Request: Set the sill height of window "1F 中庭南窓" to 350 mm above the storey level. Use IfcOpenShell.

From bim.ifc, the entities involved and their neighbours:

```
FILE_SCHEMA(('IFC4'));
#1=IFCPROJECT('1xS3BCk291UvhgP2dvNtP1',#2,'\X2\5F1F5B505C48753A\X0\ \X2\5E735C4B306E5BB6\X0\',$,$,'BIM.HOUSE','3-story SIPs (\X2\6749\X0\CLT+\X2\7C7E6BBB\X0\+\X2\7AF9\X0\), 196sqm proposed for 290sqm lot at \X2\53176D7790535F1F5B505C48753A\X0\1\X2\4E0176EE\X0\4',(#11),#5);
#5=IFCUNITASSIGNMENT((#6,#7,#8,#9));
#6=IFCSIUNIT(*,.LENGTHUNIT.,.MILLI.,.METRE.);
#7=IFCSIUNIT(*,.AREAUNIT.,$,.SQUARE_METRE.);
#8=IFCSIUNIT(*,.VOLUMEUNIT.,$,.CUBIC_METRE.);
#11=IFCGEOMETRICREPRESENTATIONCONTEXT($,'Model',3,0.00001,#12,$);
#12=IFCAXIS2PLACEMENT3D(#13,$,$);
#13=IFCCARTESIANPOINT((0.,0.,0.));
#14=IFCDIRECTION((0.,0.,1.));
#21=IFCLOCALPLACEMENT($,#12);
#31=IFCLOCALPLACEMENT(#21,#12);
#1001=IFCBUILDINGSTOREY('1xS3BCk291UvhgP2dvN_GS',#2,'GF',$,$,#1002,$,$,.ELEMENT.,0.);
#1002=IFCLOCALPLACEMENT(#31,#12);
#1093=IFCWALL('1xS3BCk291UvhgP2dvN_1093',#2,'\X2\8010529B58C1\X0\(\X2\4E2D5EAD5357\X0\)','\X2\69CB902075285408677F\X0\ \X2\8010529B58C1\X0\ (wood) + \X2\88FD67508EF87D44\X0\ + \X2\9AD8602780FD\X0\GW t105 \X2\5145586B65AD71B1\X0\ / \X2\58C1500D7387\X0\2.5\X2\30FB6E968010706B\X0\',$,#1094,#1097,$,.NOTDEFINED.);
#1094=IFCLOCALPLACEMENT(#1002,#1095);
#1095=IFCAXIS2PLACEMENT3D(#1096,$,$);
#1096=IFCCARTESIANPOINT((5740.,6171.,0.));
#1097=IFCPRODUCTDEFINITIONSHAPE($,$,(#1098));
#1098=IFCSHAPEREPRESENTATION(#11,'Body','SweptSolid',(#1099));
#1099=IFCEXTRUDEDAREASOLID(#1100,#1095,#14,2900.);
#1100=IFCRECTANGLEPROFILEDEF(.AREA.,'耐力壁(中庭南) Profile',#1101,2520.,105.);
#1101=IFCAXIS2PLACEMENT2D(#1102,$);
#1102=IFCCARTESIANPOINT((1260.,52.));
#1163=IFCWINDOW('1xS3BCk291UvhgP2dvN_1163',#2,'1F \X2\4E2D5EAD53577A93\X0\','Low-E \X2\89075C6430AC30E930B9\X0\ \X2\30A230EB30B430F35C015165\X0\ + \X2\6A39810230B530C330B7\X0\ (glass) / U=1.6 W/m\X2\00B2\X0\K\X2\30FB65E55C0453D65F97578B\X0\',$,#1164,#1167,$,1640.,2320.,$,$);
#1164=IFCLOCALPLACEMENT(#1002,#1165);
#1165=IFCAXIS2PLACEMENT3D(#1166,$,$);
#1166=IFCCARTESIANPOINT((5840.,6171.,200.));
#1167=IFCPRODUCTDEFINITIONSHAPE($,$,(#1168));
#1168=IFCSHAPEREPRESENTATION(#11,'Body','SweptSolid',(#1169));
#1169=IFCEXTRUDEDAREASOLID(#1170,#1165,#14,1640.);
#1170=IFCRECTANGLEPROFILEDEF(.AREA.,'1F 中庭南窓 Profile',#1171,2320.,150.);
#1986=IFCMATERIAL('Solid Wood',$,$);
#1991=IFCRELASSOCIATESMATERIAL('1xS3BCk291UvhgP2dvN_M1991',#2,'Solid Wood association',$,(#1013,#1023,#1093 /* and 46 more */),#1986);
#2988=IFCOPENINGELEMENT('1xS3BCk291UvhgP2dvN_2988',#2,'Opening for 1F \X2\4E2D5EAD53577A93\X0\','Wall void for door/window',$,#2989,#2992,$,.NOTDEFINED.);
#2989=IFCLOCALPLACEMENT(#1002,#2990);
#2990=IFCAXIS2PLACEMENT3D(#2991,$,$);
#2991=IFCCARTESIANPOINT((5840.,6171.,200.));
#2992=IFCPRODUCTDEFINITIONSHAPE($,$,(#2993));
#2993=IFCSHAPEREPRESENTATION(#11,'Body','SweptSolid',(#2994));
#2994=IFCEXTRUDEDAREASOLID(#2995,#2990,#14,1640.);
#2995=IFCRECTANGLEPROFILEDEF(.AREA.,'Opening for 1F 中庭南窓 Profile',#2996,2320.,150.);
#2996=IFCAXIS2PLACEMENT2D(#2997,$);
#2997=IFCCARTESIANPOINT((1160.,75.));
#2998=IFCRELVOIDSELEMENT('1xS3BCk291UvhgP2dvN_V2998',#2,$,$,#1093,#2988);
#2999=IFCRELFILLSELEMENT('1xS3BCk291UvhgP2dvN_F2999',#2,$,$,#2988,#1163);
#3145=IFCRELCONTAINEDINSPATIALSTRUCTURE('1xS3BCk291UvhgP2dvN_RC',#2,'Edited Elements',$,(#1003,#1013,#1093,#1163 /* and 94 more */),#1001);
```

```python
import numpy as np
import ifcopenshell
import ifcopenshell.api.geometry
import ifcopenshell.geom
import ifcopenshell.util.element
import ifcopenshell.util.placement
import ifcopenshell.util.shape
import ifcopenshell.util.unit

model = ifcopenshell.open("bim.ifc")
unit_scale = ifcopenshell.util.unit.calculate_unit_scale(model)

window = model.by_guid("1xS3BCk291UvhgP2dvN_1163")
opening = window.FillsVoids[0].RelatingOpeningElement
storey = ifcopenshell.util.element.get_container(window, ifc_class="IfcBuildingStorey")
level = ifcopenshell.util.placement.get_local_placement(storey.ObjectPlacement)[2, 3]

# The opening's origin need not be at the sill, so measure its lowest point.
shape = ifcopenshell.geom.create_shape(ifcopenshell.geom.settings(), opening)
bottom = ifcopenshell.util.shape.get_shape_bottom_elevation(shape, shape.geometry) / unit_scale
dz = level + 0.35 / unit_scale - bottom

shift = np.array([0.0, 0.0, dz])
# The window is not placed relative to its opening, so move both.
for product in (opening, window):
    matrix = ifcopenshell.util.placement.get_local_placement(product.ObjectPlacement)
    matrix[:3, 3] += shift
    ifcopenshell.api.geometry.edit_object_placement(model, product=product, matrix=matrix, is_si=False)

print(f"moved by {dz * unit_scale:+.3f} m")

model.write("bim_rev.ifc")
```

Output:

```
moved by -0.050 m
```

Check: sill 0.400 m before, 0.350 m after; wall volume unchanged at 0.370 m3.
